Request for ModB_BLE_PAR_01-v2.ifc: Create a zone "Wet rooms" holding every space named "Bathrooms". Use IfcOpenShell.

First a look at what the model holds.

```python
import ifcopenshell

model = ifcopenshell.open("ModB_BLE_PAR_01-v2.ifc")
print(model.schema)
seen = {}
for space in model.by_type("IfcSpace"):
    seen[space.LongName] = seen.get(space.LongName, 0) + 1
for name, count in sorted(seen.items(), key=str):
    print(count, "x", name)
print("zones:", [z.Name for z in model.by_type("IfcZone")][:20])
```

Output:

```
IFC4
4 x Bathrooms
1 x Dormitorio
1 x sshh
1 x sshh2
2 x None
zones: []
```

```python
import ifcopenshell
import ifcopenshell.api.group
import ifcopenshell.api.root

model = ifcopenshell.open("ModB_BLE_PAR_01-v2.ifc")

names = {"Bathrooms"}
spaces = [s for s in model.by_type("IfcSpace") if s.LongName in names]

zone = ifcopenshell.api.root.create_entity(model, ifc_class="IfcZone", name="Wet rooms")
ifcopenshell.api.group.assign_group(model, products=spaces, group=zone)
print(len(spaces), "spaces in", zone.Name)

model.write("ModB_BLE_PAR_01-v2_updated.ifc")
```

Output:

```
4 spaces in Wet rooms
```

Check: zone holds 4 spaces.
